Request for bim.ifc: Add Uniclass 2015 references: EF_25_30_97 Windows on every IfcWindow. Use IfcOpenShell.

First a look at what the model holds.

```python
import ifcopenshell

model = ifcopenshell.open("bim.ifc")
print(model.schema)
print("classifications:", [c.Name for c in model.by_type("IfcClassification")])
for ifc_class in ("IfcDoor", "IfcRoof", "IfcStair", "IfcWall", "IfcWindow"):
    print(ifc_class, len(model.by_type(ifc_class)))
```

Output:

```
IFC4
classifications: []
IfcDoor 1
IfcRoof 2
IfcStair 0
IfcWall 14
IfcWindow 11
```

```python
import ifcopenshell
import ifcopenshell.api.classification

model = ifcopenshell.open("bim.ifc")

system = ifcopenshell.api.classification.add_classification(model, classification="Uniclass 2015")

codes = {
    "IfcWindow": ("EF_25_30_97", "Windows"),
}
for ifc_class, (code, name) in codes.items():
    products = model.by_type(ifc_class)
    ifcopenshell.api.classification.add_reference(
        model, products=products, classification=system, identification=code, name=name
    )
    print(code, len(products))

model.write("bim_v2.ifc")
```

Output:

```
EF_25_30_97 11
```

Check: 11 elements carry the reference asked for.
